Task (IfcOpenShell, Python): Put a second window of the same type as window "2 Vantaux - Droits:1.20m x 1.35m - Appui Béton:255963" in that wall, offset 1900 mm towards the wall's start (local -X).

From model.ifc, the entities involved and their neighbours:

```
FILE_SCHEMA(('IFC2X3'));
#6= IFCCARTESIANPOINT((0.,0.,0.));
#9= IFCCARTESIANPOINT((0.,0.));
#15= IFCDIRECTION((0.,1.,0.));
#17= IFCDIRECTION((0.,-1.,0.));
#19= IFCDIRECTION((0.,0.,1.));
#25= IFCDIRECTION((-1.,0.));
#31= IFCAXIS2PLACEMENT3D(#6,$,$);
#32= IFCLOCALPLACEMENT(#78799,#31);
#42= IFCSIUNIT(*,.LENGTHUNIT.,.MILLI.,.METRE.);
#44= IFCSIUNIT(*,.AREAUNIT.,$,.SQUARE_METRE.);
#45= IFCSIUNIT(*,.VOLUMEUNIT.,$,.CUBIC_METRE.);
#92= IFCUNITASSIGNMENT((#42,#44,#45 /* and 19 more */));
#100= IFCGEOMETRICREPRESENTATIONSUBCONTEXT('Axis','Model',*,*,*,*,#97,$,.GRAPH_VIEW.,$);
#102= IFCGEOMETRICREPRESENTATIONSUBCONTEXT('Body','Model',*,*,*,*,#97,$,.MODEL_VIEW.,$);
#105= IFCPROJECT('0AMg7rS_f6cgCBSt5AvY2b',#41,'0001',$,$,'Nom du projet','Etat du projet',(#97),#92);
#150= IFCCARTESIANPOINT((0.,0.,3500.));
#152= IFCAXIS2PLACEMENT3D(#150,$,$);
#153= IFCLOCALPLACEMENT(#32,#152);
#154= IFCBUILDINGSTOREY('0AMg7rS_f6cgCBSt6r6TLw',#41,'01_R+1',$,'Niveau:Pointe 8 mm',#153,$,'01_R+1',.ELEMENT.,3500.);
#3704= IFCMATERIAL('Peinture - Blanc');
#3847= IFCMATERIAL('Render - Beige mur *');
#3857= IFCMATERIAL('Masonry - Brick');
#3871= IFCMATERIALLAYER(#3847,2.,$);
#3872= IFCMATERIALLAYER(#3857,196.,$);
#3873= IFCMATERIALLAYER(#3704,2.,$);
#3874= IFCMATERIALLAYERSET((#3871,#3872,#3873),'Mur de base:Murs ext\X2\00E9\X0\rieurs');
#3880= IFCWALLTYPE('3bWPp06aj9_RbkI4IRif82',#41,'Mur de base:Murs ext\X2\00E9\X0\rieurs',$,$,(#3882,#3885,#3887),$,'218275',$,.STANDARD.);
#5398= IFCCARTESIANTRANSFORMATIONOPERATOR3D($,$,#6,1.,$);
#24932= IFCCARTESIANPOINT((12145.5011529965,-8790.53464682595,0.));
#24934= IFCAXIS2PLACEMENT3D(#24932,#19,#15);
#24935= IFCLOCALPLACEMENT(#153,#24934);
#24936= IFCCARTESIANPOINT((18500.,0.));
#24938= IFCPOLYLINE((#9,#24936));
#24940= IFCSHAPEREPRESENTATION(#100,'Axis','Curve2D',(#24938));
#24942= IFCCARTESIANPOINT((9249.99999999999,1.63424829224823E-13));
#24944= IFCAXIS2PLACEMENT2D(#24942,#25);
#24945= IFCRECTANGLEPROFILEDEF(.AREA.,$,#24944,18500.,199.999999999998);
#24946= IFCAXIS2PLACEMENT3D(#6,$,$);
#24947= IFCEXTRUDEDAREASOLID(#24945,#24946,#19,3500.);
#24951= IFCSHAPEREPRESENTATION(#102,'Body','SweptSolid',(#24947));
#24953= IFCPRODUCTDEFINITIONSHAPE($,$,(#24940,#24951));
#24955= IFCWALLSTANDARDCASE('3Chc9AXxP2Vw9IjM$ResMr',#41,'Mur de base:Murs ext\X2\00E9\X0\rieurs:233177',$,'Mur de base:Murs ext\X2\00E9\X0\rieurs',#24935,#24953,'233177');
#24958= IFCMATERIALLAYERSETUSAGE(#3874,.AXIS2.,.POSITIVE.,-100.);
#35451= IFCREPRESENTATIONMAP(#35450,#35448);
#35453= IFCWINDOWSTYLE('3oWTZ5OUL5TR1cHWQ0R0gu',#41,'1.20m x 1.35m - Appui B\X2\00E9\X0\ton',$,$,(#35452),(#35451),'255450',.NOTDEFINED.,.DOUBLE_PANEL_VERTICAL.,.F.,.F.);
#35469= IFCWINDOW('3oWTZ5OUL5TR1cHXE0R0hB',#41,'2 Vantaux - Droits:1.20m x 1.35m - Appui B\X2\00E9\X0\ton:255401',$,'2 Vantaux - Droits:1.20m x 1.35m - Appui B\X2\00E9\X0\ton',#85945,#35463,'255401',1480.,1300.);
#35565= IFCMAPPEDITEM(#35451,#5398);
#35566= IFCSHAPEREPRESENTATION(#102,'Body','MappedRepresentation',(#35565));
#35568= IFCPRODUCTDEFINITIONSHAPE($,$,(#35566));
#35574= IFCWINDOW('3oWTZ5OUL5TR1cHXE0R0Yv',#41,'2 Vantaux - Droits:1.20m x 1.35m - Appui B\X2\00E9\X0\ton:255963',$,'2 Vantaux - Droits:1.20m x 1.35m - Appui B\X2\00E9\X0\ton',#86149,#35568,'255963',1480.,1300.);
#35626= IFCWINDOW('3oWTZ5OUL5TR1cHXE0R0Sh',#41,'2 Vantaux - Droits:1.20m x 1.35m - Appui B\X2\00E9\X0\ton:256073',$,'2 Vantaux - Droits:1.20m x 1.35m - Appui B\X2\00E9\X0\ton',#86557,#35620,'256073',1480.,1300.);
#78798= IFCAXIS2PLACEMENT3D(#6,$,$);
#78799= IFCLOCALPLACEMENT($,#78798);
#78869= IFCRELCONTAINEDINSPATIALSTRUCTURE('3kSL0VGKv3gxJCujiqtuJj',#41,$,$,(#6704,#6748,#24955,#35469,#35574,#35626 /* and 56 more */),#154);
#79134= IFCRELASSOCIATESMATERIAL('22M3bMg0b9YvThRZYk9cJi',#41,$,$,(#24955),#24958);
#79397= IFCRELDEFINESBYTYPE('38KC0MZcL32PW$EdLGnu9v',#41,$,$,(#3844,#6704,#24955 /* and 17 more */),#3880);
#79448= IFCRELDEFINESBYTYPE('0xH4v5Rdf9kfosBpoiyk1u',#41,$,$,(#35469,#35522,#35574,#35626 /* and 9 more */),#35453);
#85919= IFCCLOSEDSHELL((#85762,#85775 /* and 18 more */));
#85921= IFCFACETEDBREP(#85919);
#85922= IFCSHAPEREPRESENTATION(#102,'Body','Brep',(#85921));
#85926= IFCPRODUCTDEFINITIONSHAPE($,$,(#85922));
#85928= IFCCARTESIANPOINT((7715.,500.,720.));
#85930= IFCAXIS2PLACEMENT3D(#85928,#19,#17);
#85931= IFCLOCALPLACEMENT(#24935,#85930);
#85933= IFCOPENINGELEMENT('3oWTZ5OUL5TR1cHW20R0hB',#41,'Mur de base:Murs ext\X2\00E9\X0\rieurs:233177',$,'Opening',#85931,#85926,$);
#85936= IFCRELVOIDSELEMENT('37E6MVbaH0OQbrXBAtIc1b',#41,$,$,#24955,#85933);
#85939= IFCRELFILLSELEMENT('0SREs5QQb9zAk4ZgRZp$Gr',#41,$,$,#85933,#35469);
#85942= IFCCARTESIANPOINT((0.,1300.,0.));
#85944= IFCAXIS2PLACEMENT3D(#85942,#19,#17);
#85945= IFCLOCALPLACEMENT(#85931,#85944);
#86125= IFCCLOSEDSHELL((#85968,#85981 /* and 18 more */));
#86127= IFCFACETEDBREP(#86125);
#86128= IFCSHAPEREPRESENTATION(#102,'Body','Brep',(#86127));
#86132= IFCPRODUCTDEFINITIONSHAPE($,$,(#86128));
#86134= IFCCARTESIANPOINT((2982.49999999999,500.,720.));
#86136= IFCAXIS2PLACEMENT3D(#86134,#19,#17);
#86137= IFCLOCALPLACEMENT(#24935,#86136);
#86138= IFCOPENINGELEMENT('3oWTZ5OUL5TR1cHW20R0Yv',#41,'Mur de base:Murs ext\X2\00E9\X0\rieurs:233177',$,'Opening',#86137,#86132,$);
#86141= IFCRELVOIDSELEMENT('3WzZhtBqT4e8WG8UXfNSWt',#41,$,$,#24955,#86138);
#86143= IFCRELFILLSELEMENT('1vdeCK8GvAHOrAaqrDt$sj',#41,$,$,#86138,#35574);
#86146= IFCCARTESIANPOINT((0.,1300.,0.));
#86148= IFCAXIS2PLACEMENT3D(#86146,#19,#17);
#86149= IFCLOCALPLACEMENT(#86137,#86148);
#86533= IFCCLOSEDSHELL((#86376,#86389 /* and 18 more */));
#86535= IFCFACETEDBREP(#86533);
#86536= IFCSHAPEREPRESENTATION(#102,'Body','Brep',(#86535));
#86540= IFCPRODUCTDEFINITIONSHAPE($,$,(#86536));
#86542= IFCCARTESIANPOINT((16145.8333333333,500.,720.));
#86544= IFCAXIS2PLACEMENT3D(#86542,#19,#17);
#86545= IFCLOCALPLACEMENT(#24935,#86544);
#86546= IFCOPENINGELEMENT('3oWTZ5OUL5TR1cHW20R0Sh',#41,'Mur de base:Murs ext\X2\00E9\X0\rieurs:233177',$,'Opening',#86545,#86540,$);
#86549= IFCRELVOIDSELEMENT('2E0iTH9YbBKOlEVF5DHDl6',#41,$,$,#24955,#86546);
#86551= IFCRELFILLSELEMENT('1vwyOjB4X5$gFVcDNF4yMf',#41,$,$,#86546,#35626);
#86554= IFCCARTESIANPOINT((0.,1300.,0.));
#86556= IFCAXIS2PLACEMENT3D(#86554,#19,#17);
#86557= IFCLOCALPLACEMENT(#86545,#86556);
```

```python
import ifcopenshell
import ifcopenshell.api.feature
import ifcopenshell.api.geometry
import ifcopenshell.api.root
import ifcopenshell.geom
import ifcopenshell.util.element
import ifcopenshell.util.placement
import ifcopenshell.util.shape
import ifcopenshell.util.unit

model = ifcopenshell.open("model.ifc")
unit_scale = ifcopenshell.util.unit.calculate_unit_scale(model)
settings = ifcopenshell.geom.settings()


def volume(element):
    """Net volume in cubic metres, openings subtracted."""
    shape = ifcopenshell.geom.create_shape(settings, element)
    return ifcopenshell.util.shape.get_volume(shape.geometry)


def reuse_history(source, copy):
    """copy_class also copies each property set's owner history, people and application; keep the originals."""
    for rel in copy.IsDefinedBy:
        if rel.is_a("IfcRelDefinesByProperties") and (history := rel.RelatingPropertyDefinition.OwnerHistory):
            rel.RelatingPropertyDefinition.OwnerHistory = source.OwnerHistory
            ifcopenshell.util.element.remove_deep2(model, history)


window = model.by_guid("3oWTZ5OUL5TR1cHXE0R0Yv")
opening = window.FillsVoids[0].RelatingOpeningElement
wall = opening.VoidsElements[0].RelatingBuildingElement
before = volume(wall)
shift = ifcopenshell.util.placement.get_local_placement(wall.ObjectPlacement)[:3, 0] * -1.9 / unit_scale

# copy_class copies the void relationship, type, container and properties, but no geometry.
new_opening = ifcopenshell.api.root.copy_class(model, product=opening)
new_opening.Representation = ifcopenshell.util.element.copy_deep(
    model, opening.Representation, exclude=["IfcGeometricRepresentationContext", "IfcRepresentationMap"]
)
new_opening.Name = "Mur de base:Murs extérieurs"
new_window = ifcopenshell.api.root.copy_class(model, product=window)
new_window.Representation = ifcopenshell.util.element.copy_deep(
    model, window.Representation, exclude=["IfcGeometricRepresentationContext", "IfcRepresentationMap"]
)
new_window.Name = "2 Vantaux - Droits:1.20m x 1.35m - Appui Béton"
new_window.Tag = None
reuse_history(window, new_window)
fills = ifcopenshell.api.feature.add_filling(model, opening=new_opening, element=new_window)
fills.OwnerHistory = new_window.OwnerHistory  # required in IFC2X3

for old, new in ((opening, new_opening), (window, new_window)):
    matrix = ifcopenshell.util.placement.get_local_placement(old.ObjectPlacement)
    matrix[:3, 3] += shift
    ifcopenshell.api.geometry.edit_object_placement(model, product=new, matrix=matrix, is_si=False)

after = volume(wall)

print(f"wall volume {before:.3f} -> {after:.3f} m3")

model.write("model_edited.ifc")
```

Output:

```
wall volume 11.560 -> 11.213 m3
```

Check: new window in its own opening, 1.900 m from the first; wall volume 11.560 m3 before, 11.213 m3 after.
